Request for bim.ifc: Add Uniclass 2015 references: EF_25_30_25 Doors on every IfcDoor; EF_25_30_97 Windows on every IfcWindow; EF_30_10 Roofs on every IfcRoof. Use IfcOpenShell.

First a look at what the model holds.

```python
import ifcopenshell

model = ifcopenshell.open("bim.ifc")
print(model.schema)
print("classifications:", [c.Name for c in model.by_type("IfcClassification")])
for ifc_class in ("IfcDoor", "IfcRoof", "IfcStair", "IfcWall", "IfcWindow"):
    print(ifc_class, len(model.by_type(ifc_class)))
```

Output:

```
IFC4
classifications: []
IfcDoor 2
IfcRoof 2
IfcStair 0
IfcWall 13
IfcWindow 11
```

```python
import ifcopenshell
import ifcopenshell.api.classification

model = ifcopenshell.open("bim.ifc")

system = ifcopenshell.api.classification.add_classification(model, classification="Uniclass 2015")

codes = {
    "IfcDoor": ("EF_25_30_25", "Doors"),
    "IfcWindow": ("EF_25_30_97", "Windows"),
    "IfcRoof": ("EF_30_10", "Roofs"),
}
for ifc_class, (code, name) in codes.items():
    products = model.by_type(ifc_class)
    ifcopenshell.api.classification.add_reference(
        model, products=products, classification=system, identification=code, name=name
    )
    print(code, len(products))

model.write("bim-out.ifc")
```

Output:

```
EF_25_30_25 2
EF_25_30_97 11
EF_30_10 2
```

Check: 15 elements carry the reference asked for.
